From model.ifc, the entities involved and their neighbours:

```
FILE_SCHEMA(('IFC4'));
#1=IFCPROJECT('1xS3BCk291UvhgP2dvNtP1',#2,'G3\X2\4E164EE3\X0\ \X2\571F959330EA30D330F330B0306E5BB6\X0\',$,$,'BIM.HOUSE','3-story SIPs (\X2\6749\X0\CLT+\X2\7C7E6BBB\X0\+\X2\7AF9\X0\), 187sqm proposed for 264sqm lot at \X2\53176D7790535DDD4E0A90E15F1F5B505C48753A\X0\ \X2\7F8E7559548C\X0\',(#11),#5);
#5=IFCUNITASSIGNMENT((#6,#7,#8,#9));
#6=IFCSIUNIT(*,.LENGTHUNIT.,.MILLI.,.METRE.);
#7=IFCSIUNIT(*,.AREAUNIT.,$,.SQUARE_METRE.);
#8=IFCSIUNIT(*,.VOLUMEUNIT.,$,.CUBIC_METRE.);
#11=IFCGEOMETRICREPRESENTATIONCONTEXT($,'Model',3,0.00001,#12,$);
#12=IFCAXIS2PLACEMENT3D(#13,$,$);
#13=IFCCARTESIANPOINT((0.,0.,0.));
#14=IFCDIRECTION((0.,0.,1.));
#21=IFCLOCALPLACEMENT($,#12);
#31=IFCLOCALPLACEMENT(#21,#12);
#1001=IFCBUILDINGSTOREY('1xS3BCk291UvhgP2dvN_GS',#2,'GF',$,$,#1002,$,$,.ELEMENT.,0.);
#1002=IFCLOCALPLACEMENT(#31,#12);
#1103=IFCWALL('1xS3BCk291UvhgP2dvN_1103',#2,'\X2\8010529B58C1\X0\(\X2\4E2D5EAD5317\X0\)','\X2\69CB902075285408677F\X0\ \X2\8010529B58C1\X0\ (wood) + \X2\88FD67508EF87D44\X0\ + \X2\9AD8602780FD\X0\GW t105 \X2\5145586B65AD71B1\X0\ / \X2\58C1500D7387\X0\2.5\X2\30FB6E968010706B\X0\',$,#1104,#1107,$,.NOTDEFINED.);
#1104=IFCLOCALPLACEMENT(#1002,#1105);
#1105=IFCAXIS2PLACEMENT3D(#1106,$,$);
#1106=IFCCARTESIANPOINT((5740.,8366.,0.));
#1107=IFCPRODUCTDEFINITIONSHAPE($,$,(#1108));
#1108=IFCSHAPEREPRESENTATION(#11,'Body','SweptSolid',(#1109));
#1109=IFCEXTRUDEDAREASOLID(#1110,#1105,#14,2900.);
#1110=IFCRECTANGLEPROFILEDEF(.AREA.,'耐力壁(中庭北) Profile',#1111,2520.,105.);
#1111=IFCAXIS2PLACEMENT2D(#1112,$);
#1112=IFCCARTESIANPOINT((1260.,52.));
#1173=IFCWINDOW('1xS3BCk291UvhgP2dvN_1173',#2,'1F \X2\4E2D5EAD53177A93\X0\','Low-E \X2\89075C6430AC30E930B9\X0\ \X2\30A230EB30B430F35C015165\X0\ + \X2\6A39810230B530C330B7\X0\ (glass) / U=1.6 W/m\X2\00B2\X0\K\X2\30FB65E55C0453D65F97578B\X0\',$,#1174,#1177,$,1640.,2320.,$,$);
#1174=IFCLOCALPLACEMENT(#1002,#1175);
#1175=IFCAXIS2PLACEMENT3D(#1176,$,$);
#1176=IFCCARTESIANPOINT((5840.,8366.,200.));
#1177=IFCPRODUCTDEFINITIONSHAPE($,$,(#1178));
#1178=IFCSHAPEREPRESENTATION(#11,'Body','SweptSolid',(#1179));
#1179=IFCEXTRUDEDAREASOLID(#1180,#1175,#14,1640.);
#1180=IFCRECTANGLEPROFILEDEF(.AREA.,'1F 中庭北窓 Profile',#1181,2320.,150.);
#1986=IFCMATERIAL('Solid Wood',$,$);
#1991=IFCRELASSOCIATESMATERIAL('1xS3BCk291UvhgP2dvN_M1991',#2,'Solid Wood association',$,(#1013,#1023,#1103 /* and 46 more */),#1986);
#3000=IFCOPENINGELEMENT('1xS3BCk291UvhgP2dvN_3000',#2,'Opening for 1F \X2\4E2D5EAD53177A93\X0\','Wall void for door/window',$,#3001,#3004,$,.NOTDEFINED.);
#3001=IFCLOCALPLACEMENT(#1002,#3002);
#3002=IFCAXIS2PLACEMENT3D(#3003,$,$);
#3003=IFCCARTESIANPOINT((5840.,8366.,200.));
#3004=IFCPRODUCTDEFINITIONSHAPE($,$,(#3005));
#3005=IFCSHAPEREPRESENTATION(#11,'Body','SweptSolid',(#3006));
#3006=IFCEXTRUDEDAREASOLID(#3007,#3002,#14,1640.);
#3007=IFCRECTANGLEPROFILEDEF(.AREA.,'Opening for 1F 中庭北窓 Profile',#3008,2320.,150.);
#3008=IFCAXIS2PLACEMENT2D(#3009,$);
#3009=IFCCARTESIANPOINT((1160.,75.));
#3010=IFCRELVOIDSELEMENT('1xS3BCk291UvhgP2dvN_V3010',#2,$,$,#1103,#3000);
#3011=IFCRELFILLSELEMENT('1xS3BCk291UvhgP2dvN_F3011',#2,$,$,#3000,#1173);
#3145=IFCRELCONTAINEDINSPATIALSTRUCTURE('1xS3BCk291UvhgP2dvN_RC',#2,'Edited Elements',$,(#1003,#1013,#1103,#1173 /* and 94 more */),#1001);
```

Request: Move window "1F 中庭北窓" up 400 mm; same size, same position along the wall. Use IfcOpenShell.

```python
import numpy as np
import ifcopenshell
import ifcopenshell.api.geometry
import ifcopenshell.util.placement
import ifcopenshell.util.unit

model = ifcopenshell.open("model.ifc")
unit_scale = ifcopenshell.util.unit.calculate_unit_scale(model)

window = model.by_id(1173)
opening = window.FillsVoids[0].RelatingOpeningElement
dz = 0.4 / unit_scale

shift = np.array([0.0, 0.0, dz])
# The window is not placed relative to its opening, so move both.
for product in (opening, window):
    matrix = ifcopenshell.util.placement.get_local_placement(product.ObjectPlacement)
    matrix[:3, 3] += shift
    ifcopenshell.api.geometry.edit_object_placement(model, product=product, matrix=matrix, is_si=False)

print(f"moved by {dz * unit_scale:+.3f} m")

model.write("model-out.ifc")
```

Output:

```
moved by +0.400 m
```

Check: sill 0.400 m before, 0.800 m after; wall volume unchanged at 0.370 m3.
